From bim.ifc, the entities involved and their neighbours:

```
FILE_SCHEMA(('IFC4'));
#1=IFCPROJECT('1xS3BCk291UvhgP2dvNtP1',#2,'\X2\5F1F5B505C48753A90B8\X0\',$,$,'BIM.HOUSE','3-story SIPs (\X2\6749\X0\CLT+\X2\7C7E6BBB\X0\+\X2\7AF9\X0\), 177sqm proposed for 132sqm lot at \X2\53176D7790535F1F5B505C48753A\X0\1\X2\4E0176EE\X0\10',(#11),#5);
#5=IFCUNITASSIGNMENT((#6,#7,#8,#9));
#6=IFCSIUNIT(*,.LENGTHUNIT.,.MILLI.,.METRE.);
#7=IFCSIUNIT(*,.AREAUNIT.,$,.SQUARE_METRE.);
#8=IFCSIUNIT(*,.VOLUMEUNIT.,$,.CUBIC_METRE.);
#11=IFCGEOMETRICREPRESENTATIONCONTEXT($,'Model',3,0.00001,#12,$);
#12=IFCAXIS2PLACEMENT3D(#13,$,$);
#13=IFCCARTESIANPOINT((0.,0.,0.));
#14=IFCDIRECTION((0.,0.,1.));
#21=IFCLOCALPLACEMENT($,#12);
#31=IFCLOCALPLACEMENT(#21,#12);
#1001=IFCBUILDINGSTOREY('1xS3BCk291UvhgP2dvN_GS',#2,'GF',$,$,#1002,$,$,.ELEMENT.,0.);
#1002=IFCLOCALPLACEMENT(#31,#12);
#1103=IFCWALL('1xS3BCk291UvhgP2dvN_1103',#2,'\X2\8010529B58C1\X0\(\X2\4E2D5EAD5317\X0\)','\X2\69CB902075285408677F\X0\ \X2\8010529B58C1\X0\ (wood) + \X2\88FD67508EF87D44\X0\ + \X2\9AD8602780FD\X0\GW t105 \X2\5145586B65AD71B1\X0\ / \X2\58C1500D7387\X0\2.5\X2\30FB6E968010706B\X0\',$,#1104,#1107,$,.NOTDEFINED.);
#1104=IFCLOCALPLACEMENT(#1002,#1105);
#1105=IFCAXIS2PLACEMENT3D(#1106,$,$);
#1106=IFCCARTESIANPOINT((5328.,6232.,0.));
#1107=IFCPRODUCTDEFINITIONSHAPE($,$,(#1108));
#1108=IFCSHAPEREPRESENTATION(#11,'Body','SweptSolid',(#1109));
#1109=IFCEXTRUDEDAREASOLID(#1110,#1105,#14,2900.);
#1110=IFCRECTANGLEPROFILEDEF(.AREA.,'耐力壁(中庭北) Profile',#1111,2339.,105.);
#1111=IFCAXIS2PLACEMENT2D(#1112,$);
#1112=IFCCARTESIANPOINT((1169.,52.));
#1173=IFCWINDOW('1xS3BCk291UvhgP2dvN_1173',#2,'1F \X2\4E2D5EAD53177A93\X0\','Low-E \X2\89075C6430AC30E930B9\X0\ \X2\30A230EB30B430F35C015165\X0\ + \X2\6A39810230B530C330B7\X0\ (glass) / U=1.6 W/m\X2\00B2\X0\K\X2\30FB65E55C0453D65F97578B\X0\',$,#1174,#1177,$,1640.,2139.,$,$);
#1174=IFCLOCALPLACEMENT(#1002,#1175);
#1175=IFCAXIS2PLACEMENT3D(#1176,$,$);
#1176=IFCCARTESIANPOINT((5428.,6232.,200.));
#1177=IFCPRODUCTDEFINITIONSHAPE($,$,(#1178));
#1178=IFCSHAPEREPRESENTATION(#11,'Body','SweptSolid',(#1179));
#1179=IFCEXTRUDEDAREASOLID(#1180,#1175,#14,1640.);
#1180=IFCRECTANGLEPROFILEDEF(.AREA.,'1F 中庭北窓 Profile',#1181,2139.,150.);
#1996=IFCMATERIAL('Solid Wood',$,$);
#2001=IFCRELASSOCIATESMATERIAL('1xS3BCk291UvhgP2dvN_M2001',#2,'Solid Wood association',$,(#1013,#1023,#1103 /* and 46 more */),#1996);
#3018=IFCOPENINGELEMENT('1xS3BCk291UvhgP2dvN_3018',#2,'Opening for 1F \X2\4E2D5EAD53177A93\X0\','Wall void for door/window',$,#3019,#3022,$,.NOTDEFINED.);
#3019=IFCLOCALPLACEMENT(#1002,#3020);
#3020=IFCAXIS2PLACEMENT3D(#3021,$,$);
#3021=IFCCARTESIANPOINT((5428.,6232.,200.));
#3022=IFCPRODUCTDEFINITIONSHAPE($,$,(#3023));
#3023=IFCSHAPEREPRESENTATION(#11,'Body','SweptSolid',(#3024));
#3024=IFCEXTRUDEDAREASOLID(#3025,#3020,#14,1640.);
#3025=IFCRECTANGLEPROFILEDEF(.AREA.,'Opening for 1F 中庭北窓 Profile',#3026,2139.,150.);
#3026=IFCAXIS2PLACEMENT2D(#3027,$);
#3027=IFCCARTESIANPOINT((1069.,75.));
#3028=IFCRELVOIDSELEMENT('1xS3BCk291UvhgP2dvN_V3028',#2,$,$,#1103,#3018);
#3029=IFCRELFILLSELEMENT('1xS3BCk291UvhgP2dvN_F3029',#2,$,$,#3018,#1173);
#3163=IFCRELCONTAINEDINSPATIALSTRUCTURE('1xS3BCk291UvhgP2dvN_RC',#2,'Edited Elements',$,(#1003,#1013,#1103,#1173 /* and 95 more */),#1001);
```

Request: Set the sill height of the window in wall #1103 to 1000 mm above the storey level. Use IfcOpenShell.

```python
import numpy as np
import ifcopenshell
import ifcopenshell.api.geometry
import ifcopenshell.geom
import ifcopenshell.util.element
import ifcopenshell.util.placement
import ifcopenshell.util.shape
import ifcopenshell.util.unit

model = ifcopenshell.open("bim.ifc")
unit_scale = ifcopenshell.util.unit.calculate_unit_scale(model)

window = model.by_id(1173)
opening = window.FillsVoids[0].RelatingOpeningElement
storey = ifcopenshell.util.element.get_container(window, ifc_class="IfcBuildingStorey")
level = ifcopenshell.util.placement.get_local_placement(storey.ObjectPlacement)[2, 3]

# The opening's origin need not be at the sill, so measure its lowest point.
shape = ifcopenshell.geom.create_shape(ifcopenshell.geom.settings(), opening)
bottom = ifcopenshell.util.shape.get_shape_bottom_elevation(shape, shape.geometry) / unit_scale
dz = level + 1 / unit_scale - bottom

shift = np.array([0.0, 0.0, dz])
# The window is not placed relative to its opening, so move both.
for product in (opening, window):
    matrix = ifcopenshell.util.placement.get_local_placement(product.ObjectPlacement)
    matrix[:3, 3] += shift
    ifcopenshell.api.geometry.edit_object_placement(model, product=product, matrix=matrix, is_si=False)

print(f"moved by {dz * unit_scale:+.3f} m")

model.write("bim_edited.ifc")
```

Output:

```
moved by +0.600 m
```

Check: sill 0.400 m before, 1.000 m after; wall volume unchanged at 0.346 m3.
